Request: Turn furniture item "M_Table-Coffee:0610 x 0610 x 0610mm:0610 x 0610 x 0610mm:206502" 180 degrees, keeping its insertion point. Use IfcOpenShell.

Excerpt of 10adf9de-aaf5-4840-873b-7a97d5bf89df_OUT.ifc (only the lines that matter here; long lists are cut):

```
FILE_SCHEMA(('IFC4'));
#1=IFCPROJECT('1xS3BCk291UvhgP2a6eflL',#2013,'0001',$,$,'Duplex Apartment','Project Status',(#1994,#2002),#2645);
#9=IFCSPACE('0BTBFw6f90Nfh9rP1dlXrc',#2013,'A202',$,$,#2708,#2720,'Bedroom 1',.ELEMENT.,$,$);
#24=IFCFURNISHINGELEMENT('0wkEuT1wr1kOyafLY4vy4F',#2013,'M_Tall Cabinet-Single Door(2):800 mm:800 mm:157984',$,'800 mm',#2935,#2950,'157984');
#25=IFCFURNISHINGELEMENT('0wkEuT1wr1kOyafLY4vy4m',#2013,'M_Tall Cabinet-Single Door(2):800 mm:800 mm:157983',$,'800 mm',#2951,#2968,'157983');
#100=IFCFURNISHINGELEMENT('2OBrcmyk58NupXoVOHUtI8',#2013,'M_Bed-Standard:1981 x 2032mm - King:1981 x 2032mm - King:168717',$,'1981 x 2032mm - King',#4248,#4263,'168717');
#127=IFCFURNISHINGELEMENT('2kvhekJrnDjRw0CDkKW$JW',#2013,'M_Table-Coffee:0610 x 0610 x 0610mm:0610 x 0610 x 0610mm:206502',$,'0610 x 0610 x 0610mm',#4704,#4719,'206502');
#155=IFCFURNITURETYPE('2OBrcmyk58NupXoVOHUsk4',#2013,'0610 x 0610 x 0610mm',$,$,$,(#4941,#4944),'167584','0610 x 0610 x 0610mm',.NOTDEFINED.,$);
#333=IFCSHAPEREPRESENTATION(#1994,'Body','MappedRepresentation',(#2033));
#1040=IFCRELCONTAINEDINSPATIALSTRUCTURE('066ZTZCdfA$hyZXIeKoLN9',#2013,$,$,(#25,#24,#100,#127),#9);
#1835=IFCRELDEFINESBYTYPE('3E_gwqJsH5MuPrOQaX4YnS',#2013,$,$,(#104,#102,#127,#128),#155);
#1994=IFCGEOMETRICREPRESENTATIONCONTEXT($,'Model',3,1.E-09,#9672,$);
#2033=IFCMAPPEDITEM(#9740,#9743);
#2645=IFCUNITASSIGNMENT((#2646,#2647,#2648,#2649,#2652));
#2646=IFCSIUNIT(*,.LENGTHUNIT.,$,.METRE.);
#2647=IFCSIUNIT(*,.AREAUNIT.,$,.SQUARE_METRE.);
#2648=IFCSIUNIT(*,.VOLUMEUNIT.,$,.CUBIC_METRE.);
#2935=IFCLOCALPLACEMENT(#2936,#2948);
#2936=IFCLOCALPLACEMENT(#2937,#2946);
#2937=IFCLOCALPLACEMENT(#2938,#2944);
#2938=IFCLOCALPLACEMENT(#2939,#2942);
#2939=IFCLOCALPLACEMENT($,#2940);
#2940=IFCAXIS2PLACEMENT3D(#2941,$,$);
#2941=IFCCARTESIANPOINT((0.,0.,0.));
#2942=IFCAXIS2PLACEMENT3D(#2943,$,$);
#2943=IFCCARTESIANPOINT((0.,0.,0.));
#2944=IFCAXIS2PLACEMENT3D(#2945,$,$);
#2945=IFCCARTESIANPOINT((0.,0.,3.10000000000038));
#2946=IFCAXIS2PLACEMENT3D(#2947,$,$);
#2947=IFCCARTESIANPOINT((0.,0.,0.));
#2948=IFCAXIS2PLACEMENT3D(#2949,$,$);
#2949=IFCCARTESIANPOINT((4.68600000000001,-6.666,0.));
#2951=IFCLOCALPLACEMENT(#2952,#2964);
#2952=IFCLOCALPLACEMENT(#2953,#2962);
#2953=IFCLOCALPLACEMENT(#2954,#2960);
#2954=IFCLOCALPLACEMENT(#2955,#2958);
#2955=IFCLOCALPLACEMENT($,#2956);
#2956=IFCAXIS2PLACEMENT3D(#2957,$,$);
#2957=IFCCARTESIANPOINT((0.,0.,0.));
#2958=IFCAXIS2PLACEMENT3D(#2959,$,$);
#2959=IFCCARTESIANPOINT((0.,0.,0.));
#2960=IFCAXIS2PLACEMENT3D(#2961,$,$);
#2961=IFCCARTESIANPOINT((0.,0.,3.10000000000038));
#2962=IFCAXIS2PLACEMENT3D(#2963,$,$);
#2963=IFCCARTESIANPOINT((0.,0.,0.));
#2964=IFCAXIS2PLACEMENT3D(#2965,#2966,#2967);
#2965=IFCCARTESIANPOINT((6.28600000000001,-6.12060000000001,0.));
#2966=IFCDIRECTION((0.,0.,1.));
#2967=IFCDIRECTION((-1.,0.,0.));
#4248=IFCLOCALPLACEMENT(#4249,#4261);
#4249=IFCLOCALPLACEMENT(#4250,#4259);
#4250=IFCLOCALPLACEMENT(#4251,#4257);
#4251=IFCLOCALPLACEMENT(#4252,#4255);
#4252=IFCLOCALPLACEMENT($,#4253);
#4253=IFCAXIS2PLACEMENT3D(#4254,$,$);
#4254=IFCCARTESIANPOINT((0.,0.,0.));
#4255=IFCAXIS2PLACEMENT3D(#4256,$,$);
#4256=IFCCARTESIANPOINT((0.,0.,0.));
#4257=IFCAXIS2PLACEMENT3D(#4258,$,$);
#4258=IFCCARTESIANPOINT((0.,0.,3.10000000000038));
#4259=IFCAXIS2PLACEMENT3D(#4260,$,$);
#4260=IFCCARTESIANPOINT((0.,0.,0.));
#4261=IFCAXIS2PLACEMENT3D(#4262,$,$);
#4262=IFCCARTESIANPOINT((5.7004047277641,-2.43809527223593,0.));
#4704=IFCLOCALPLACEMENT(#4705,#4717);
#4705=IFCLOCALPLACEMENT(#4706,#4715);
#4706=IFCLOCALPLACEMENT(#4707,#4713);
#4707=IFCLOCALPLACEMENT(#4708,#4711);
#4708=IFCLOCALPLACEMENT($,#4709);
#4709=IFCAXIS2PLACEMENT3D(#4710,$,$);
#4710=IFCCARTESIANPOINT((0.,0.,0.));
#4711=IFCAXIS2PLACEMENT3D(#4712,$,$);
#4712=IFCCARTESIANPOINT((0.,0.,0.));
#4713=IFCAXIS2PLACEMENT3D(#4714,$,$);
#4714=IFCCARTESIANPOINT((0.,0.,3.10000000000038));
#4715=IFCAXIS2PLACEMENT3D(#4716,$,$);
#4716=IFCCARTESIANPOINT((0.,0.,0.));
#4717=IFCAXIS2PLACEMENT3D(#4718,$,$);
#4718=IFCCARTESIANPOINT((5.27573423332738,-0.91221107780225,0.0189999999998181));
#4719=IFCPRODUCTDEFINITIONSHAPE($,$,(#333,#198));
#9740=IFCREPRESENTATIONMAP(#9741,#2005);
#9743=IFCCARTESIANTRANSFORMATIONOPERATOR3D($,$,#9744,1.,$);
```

```python
import ifcopenshell
import ifcopenshell.api.geometry
import ifcopenshell.util.placement

model = ifcopenshell.open("10adf9de-aaf5-4840-873b-7a97d5bf89df_OUT.ifc")

item = model.by_id(127)
matrix = ifcopenshell.util.placement.get_local_placement(item.ObjectPlacement)
matrix = matrix @ ifcopenshell.util.placement.rotation(180, "Z")
ifcopenshell.api.geometry.edit_object_placement(model, product=item, matrix=matrix, is_si=False)

print(ifcopenshell.util.placement.get_local_placement(item.ObjectPlacement).round(3) + 0.0)

model.write("10adf9de-aaf5-4840-873b-7a97d5bf89df_OUT_edited.ifc")
```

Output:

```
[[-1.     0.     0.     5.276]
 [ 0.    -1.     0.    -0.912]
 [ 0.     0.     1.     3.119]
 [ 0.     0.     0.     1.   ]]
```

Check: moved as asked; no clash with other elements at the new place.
